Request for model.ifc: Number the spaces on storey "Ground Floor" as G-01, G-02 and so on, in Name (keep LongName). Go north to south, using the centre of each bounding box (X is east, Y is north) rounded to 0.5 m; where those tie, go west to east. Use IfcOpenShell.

First a look at what the model holds.

```python
import ifcopenshell
import ifcopenshell.util.element
import ifcopenshell.util.placement

model = ifcopenshell.open("model.ifc")
print(model.schema)
storey = next(s for s in model.by_type("IfcBuildingStorey") if s.Name == "Ground Floor")
spaces = [e for e in ifcopenshell.util.element.get_decomposition(storey) if e.is_a("IfcSpace")]
for e in sorted(spaces, key=lambda e: e.id()):
    origin = ifcopenshell.util.placement.get_local_placement(e.ObjectPlacement)[:3, 3]
    print(e.id(), e.Name, e.LongName, origin.round(2) + 0.0, sep=" | ")
```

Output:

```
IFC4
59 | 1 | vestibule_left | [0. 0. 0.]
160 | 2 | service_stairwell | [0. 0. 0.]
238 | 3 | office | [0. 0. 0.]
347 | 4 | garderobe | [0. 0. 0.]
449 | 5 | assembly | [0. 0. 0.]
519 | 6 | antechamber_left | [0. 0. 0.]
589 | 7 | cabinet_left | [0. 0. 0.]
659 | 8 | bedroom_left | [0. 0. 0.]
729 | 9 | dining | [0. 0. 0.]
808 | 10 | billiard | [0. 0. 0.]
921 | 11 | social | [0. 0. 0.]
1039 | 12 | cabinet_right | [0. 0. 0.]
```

```python
import ifcopenshell
import ifcopenshell.geom
import ifcopenshell.util.element
import ifcopenshell.util.shape

model = ifcopenshell.open("model.ifc")
settings = ifcopenshell.geom.settings()
settings.set("use-world-coords", True)


def centre(element):
    shape = ifcopenshell.geom.create_shape(settings, element)
    return ifcopenshell.util.shape.get_bbox_centroid(shape.geometry)


storey = next(s for s in model.by_type("IfcBuildingStorey") if s.Name == "Ground Floor")
spaces = [e for e in ifcopenshell.util.element.get_decomposition(storey) if e.is_a("IfcSpace")]

# Insertion points can sit at a corner or the storey origin, so sort by the geometry (in metres).
centres = {e: centre(e) for e in spaces}
spaces.sort(key=lambda e: (-round(centres[e][1] / 0.5), centres[e][0]))

for i, e in enumerate(spaces, start=1):
    number = f"G-{i:02d}"
    e.Name = number
    print(e.id(), number)

model.write("model_rev.ifc")
```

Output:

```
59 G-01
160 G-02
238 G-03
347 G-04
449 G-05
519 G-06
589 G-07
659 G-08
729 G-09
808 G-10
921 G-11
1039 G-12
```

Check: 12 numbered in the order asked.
